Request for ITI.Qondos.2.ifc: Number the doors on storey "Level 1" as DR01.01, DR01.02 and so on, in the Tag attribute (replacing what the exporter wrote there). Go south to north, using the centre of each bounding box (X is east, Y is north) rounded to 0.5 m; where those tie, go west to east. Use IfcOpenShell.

First a look at what the model holds.

```python
import ifcopenshell
import ifcopenshell.util.element
import ifcopenshell.util.placement

model = ifcopenshell.open("ITI.Qondos.2.ifc")
print(model.schema)
storey = next(s for s in model.by_type("IfcBuildingStorey") if s.Name == "Level 1")
doors = [e for e in ifcopenshell.util.element.get_decomposition(storey) if e.is_a("IfcDoor")]
for e in sorted(doors, key=lambda e: e.id()):
    origin = ifcopenshell.util.placement.get_local_placement(e.ObjectPlacement)[:3, 3]
    print(e.id(), e.Tag, e.Name, origin.round(2) + 0.0, sep=" | ")
```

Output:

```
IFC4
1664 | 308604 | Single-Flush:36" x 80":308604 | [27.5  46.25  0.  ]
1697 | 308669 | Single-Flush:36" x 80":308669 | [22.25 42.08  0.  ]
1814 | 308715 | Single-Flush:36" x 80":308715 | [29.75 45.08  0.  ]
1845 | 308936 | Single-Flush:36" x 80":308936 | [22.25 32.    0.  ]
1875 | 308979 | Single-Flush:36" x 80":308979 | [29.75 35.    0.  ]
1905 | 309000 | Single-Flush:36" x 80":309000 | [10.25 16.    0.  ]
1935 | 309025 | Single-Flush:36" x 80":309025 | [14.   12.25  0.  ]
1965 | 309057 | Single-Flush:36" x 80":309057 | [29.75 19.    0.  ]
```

```python
import ifcopenshell
import ifcopenshell.geom
import ifcopenshell.util.element
import ifcopenshell.util.shape

model = ifcopenshell.open("ITI.Qondos.2.ifc")
settings = ifcopenshell.geom.settings()
settings.set("use-world-coords", True)


def centre(element):
    shape = ifcopenshell.geom.create_shape(settings, element)
    return ifcopenshell.util.shape.get_bbox_centroid(shape.geometry)


storey = next(s for s in model.by_type("IfcBuildingStorey") if s.Name == "Level 1")
doors = [e for e in ifcopenshell.util.element.get_decomposition(storey) if e.is_a("IfcDoor")]

# Insertion points can sit at a corner or the storey origin, so sort by the geometry (in metres).
centres = {e: centre(e) for e in doors}
doors.sort(key=lambda e: (round(centres[e][1] / 0.5), centres[e][0]))

for i, e in enumerate(doors, start=1):
    number = f"DR01.{i:02d}"
    e.Tag = number
    print(e.id(), number)

model.write("ITI.Qondos.2_edited.ifc")
```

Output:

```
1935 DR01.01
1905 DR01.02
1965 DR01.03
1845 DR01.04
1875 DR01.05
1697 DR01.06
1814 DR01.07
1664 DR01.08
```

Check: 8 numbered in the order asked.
